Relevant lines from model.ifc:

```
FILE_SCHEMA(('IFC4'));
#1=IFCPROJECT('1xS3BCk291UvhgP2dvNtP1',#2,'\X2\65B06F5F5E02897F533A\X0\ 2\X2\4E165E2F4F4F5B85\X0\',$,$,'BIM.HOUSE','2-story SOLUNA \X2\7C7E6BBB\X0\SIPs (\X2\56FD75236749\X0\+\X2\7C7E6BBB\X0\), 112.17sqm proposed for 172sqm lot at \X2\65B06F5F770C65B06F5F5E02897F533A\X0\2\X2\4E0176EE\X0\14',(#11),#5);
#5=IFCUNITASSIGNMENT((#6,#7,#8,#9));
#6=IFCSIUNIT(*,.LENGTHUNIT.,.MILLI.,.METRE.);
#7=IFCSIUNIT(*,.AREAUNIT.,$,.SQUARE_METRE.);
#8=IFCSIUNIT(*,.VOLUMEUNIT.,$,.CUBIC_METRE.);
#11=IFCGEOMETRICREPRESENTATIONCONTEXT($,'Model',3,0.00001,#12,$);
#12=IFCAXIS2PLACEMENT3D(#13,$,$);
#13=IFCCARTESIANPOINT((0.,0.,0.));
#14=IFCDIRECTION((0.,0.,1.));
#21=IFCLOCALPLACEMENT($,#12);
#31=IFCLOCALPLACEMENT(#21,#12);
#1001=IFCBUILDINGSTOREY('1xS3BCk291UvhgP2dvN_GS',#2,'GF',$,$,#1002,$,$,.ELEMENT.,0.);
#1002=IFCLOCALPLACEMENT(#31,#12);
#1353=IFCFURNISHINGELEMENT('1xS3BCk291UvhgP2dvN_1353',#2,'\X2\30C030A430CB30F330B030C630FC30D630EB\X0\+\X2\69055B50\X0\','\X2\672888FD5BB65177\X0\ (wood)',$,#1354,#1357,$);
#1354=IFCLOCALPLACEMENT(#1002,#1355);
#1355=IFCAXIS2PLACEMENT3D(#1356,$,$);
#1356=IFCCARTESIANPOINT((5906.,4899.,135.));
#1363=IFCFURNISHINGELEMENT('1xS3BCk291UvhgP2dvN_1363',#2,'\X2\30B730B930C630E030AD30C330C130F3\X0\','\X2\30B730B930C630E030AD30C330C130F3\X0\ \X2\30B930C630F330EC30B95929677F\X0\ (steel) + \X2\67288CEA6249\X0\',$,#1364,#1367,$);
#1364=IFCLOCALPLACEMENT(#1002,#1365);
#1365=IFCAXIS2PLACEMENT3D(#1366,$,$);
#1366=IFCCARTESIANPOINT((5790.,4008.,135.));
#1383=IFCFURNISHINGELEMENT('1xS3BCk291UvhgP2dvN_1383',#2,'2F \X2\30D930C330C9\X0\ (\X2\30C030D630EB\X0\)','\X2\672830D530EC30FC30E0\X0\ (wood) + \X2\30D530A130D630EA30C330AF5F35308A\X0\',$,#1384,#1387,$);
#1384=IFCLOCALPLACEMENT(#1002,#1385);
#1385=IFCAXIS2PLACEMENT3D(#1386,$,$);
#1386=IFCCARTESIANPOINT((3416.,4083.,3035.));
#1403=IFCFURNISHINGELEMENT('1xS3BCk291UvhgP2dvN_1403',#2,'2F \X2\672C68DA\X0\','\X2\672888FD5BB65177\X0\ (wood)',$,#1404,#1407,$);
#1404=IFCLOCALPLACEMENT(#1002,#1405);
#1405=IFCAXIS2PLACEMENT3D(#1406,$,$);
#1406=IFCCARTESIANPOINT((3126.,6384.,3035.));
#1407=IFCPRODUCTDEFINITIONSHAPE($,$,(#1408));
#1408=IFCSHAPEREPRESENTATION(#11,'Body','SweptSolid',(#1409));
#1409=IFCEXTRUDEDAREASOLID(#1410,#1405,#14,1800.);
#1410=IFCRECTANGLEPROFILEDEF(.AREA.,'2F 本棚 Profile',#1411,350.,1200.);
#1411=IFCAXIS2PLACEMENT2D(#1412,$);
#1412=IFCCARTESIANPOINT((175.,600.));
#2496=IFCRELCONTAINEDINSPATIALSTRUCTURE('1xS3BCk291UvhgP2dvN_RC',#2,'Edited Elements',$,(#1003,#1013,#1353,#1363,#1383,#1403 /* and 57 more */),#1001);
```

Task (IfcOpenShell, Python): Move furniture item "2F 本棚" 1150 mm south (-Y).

```python
import ifcopenshell
import ifcopenshell.api.geometry
import ifcopenshell.util.placement
import ifcopenshell.util.unit

model = ifcopenshell.open("model.ifc")
unit_scale = ifcopenshell.util.unit.calculate_unit_scale(model)

item = model.by_guid("1xS3BCk291UvhgP2dvN_1403")
matrix = ifcopenshell.util.placement.get_local_placement(item.ObjectPlacement)
matrix[1, 3] -= 1.15 / unit_scale
ifcopenshell.api.geometry.edit_object_placement(model, product=item, matrix=matrix, is_si=False)

print(ifcopenshell.util.placement.get_local_placement(item.ObjectPlacement).round(3) + 0.0)

model.write("model_v2.ifc")
```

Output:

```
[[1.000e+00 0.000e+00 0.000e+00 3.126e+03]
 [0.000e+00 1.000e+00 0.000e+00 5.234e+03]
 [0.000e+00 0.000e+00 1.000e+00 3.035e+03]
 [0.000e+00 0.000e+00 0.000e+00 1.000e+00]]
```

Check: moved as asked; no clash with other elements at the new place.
